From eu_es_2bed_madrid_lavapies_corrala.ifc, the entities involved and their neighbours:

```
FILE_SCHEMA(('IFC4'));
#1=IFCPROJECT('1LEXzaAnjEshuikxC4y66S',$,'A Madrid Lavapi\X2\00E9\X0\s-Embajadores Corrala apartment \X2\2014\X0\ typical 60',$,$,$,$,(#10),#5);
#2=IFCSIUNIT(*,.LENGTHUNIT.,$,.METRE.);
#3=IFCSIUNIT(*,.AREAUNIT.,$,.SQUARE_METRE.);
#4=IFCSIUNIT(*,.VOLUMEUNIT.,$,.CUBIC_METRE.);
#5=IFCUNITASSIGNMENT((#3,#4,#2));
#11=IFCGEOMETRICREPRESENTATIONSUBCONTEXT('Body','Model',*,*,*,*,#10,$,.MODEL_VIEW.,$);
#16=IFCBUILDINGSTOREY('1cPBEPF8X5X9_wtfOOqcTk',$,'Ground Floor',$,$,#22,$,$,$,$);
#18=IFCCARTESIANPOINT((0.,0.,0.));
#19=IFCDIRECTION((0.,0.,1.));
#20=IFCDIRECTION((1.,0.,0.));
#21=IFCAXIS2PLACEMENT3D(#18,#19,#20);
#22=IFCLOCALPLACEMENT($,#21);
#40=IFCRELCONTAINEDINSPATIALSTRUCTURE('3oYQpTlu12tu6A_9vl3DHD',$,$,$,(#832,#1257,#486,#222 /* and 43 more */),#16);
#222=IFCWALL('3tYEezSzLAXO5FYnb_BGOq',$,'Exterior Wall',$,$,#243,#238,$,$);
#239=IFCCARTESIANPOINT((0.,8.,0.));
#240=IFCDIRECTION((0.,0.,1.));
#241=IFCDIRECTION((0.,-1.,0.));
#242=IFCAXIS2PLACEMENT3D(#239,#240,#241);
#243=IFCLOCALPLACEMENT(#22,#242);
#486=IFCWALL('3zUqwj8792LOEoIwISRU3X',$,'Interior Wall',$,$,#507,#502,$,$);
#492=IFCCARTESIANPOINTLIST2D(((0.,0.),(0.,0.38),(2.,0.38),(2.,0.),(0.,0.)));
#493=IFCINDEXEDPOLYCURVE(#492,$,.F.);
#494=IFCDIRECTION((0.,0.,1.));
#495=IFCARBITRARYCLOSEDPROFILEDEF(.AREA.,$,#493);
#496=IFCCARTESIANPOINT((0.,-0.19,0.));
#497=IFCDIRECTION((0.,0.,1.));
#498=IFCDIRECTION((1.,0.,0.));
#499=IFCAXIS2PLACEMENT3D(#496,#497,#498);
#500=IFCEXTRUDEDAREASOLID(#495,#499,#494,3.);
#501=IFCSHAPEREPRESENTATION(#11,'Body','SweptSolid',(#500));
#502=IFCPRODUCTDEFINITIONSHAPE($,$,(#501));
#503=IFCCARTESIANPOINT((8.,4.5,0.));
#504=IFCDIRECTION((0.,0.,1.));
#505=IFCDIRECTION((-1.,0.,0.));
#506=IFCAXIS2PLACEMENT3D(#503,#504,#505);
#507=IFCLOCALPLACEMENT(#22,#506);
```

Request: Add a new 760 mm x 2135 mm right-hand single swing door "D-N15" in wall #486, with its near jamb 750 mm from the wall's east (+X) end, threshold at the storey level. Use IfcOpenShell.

```python
import numpy as np
import ifcopenshell
import ifcopenshell.api.feature
import ifcopenshell.api.geometry
import ifcopenshell.api.root
import ifcopenshell.api.spatial
import ifcopenshell.geom
import ifcopenshell.util.element
import ifcopenshell.util.placement
import ifcopenshell.util.representation
import ifcopenshell.util.shape
import ifcopenshell.util.unit

model = ifcopenshell.open("eu_es_2bed_madrid_lavapies_corrala.ifc")
unit_scale = ifcopenshell.util.unit.calculate_unit_scale(model)
settings = ifcopenshell.geom.settings()


def volume(element):
    """Net volume in cubic metres, openings subtracted."""
    shape = ifcopenshell.geom.create_shape(settings, element)
    return ifcopenshell.util.shape.get_volume(shape.geometry)


wall = model.by_guid("3zUqwj8792LOEoIwISRU3X")
storey = ifcopenshell.util.element.get_container(wall, ifc_class="IfcBuildingStorey")
context = ifcopenshell.util.representation.get_context(model, "Model", "Body", "MODEL_VIEW")
before = volume(wall)

width, height, from_end, sill = 0.76, 2.135, 0.75, 0.0  # metres

# The wall runs along its own X axis, and the end named is its -X end.
wall_shape = ifcopenshell.geom.create_shape(settings, wall)
x, y, z = ifcopenshell.util.shape.get_vertices(wall_shape.geometry).T
start = x.min() + from_end
face, thickness = float(y.min()), float(y.max() - y.min())
wall_matrix = ifcopenshell.util.placement.get_local_placement(wall.ObjectPlacement)
level = ifcopenshell.util.placement.get_local_placement(storey.ObjectPlacement)[2, 3]


def in_wall(x, y):
    """Placement at x, y metres in the wall's axes, at sill height."""
    matrix = wall_matrix.copy()
    matrix[:, 3] = wall_matrix @ np.array([x / unit_scale, y / unit_scale, 0.0, 1.0])
    matrix[2, 3] = level + sill / unit_scale
    return matrix


# Opening: a box that overshoots both wall faces by 50 mm.
opening = ifcopenshell.api.root.create_entity(model, ifc_class="IfcOpeningElement", predefined_type="OPENING")
box = ifcopenshell.api.geometry.add_wall_representation(
    model, context=context, length=width, height=height, thickness=thickness + 0.1
)
ifcopenshell.api.geometry.assign_representation(model, product=opening, representation=box)
ifcopenshell.api.geometry.edit_object_placement(model, product=opening, matrix=in_wall(start, face - 0.05), is_si=False)
ifcopenshell.api.feature.add_feature(model, feature=opening, element=wall)

door = ifcopenshell.api.root.create_entity(model, ifc_class="IfcDoor", name="D-N15", predefined_type="DOOR")
door.OverallWidth, door.OverallHeight = width / unit_scale, height / unit_scale
door.OperationType = "SINGLE_SWING_RIGHT"
body = ifcopenshell.api.geometry.add_door_representation(
    model,
    context=context,
    overall_width=door.OverallWidth,
    overall_height=door.OverallHeight,
    operation_type="SINGLE_SWING_RIGHT",
    lining_properties={"LiningDepth": thickness / unit_scale, "ThresholdDepth": thickness / unit_scale},
)
ifcopenshell.api.geometry.assign_representation(model, product=door, representation=body)
ifcopenshell.api.spatial.assign_container(model, products=[door], relating_structure=storey)
ifcopenshell.api.feature.add_filling(model, opening=opening, element=door)

# The lining spans the wall, so the door starts at the wall face.
ifcopenshell.api.geometry.edit_object_placement(model, product=door, matrix=in_wall(start, face), is_si=False)

after = volume(wall)

print(f"wall volume {before:.3f} -> {after:.3f} m3")

model.write("eu_es_2bed_madrid_lavapies_corrala_edited.ifc")
```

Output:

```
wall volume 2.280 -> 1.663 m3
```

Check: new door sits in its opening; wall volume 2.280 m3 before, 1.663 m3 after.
